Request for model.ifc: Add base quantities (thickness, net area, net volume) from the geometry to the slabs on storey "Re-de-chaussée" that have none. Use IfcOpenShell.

First a look at what the model holds.

```python
import ifcopenshell
import ifcopenshell.util.element
import ifcopenshell.util.unit

model = ifcopenshell.open("model.ifc")
print(model.schema)
for unit_type in ("LENGTHUNIT", "AREAUNIT", "VOLUMEUNIT"):
    print(unit_type, ifcopenshell.util.unit.calculate_unit_scale(model, unit_type))
storey = next(s for s in model.by_type("IfcBuildingStorey") if s.Name == "Re-de-chaussée")
slabs = [e for e in ifcopenshell.util.element.get_decomposition(storey) if e.is_a("IfcSlab")]
for e in sorted(slabs, key=lambda e: e.id()):
    print(e.id(), e.is_a(), e.Name, list(ifcopenshell.util.element.get_psets(e, qtos_only=True)), sep=" | ")
```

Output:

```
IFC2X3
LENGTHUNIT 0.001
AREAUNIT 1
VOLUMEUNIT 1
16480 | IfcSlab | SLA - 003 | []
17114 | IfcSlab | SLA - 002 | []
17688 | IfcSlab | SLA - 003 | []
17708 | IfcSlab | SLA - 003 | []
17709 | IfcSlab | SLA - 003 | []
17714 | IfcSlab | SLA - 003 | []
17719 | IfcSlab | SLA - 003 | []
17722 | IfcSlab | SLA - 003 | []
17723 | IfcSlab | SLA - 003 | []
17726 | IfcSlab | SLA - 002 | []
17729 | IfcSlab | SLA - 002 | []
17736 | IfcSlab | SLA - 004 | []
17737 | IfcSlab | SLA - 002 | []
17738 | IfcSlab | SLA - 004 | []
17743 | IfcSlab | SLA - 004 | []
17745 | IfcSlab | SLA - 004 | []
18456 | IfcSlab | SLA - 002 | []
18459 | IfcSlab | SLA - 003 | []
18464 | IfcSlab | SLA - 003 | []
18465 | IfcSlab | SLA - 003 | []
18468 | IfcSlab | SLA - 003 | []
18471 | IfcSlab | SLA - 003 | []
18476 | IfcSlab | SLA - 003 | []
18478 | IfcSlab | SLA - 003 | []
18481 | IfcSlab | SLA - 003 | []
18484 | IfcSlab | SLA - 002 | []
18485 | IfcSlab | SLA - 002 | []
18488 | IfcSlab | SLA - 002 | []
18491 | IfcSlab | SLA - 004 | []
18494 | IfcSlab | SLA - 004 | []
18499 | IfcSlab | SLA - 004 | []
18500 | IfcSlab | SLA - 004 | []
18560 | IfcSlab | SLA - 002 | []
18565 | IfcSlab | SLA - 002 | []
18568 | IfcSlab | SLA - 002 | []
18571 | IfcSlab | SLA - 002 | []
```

```python
import ifcopenshell
import ifcopenshell.api.pset
import ifcopenshell.geom
import ifcopenshell.util.element
import ifcopenshell.util.shape
import ifcopenshell.util.unit

model = ifcopenshell.open("model.ifc")
unit_scale = ifcopenshell.util.unit.calculate_unit_scale(model)
area_scale = ifcopenshell.util.unit.calculate_unit_scale(model, "AREAUNIT")
volume_scale = ifcopenshell.util.unit.calculate_unit_scale(model, "VOLUMEUNIT")
settings = ifcopenshell.geom.settings()

storey = next(s for s in model.by_type("IfcBuildingStorey") if s.Name == "Re-de-chaussée")
slabs = [e for e in ifcopenshell.util.element.get_decomposition(storey) if e.is_a("IfcSlab")]

for e in sorted(slabs, key=lambda e: e.id()):
    if ifcopenshell.util.element.get_psets(e, qtos_only=True, should_inherit=False):
        continue
    # Geometry comes back in metres, in the element's own axes.
    shape = ifcopenshell.geom.create_shape(settings, e)
    values = {
        "Width": ifcopenshell.util.shape.get_z(shape.geometry) / unit_scale,
        "NetArea": ifcopenshell.util.shape.get_footprint_area(shape.geometry) / area_scale,
        "NetVolume": ifcopenshell.util.shape.get_volume(shape.geometry) / volume_scale,
    }
    qto = ifcopenshell.api.pset.add_qto(model, product=e, name="BaseQuantities")
    ifcopenshell.api.pset.edit_qto(model, qto=qto, properties=values)
    print(e.id(), {k: round(v, 3) for k, v in values.items()})

model.write("model_v2.ifc")
```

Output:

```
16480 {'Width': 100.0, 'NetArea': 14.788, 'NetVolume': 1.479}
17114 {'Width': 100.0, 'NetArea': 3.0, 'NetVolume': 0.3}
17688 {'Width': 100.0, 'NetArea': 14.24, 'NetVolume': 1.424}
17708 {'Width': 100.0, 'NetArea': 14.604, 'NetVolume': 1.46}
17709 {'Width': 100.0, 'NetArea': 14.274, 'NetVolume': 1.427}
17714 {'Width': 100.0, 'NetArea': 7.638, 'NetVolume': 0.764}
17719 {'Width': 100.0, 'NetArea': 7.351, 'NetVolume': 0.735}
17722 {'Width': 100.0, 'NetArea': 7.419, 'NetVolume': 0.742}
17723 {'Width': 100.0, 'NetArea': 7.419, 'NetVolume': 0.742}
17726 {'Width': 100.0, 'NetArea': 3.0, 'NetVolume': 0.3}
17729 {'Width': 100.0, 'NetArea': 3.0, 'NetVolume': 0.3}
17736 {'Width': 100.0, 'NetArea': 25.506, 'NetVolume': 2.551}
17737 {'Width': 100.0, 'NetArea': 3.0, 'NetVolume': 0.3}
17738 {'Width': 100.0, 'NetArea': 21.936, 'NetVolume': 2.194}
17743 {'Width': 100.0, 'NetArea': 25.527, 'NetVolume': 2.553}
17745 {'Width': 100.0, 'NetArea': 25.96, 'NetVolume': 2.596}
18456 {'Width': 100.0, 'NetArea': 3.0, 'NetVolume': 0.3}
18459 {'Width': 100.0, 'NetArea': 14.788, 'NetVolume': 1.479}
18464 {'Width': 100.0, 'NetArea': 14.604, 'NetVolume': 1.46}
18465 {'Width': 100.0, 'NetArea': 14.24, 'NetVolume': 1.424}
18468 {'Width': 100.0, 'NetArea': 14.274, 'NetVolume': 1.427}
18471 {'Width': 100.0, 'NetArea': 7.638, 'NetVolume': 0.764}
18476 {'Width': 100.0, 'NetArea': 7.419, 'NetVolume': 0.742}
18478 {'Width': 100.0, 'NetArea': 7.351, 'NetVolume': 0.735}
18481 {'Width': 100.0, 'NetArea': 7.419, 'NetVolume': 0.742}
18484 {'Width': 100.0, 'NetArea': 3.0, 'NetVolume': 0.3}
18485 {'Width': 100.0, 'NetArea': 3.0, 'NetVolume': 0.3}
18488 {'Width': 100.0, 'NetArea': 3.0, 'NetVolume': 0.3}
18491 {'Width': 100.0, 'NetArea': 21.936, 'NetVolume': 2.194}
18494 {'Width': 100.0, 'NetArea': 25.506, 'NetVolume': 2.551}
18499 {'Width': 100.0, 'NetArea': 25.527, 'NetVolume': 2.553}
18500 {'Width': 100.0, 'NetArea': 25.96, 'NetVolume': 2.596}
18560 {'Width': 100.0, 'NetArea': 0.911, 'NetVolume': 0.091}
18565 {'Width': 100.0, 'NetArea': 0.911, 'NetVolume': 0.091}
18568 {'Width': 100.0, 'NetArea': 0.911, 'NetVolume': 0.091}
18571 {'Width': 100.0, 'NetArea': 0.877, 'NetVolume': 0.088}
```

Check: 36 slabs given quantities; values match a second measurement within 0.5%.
